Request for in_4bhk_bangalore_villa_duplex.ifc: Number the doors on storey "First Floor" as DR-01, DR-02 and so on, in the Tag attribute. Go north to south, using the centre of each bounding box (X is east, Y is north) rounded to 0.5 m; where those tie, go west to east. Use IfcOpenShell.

First a look at what the model holds.

```python
import ifcopenshell
import ifcopenshell.util.element
import ifcopenshell.util.placement

model = ifcopenshell.open("in_4bhk_bangalore_villa_duplex.ifc")
print(model.schema)
storey = next(s for s in model.by_type("IfcBuildingStorey") if s.Name == "First Floor")
doors = [e for e in ifcopenshell.util.element.get_decomposition(storey) if e.is_a("IfcDoor")]
for e in sorted(doors, key=lambda e: e.id()):
    origin = ifcopenshell.util.placement.get_local_placement(e.ObjectPlacement)[:3, 3]
    print(e.id(), e.Tag, e.Name, origin.round(2) + 0.0, sep=" | ")
```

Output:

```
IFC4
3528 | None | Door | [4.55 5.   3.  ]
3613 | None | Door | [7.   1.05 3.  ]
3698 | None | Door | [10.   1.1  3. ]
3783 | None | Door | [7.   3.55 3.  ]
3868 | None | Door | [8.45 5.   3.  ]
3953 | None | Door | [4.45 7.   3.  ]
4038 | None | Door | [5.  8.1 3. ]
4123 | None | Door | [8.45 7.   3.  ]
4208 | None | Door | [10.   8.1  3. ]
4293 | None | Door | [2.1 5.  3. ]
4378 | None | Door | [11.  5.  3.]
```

```python
import ifcopenshell
import ifcopenshell.geom
import ifcopenshell.util.element
import ifcopenshell.util.shape

model = ifcopenshell.open("in_4bhk_bangalore_villa_duplex.ifc")
settings = ifcopenshell.geom.settings()
settings.set("use-world-coords", True)


def centre(element):
    shape = ifcopenshell.geom.create_shape(settings, element)
    return ifcopenshell.util.shape.get_bbox_centroid(shape.geometry)


storey = next(s for s in model.by_type("IfcBuildingStorey") if s.Name == "First Floor")
doors = [e for e in ifcopenshell.util.element.get_decomposition(storey) if e.is_a("IfcDoor")]

# Insertion points can sit at a corner or the storey origin, so sort by the geometry (in metres).
centres = {e: centre(e) for e in doors}
doors.sort(key=lambda e: (-round(centres[e][1] / 0.5), centres[e][0]))

for i, e in enumerate(doors, start=1):
    number = f"DR-{i:02d}"
    e.Tag = number
    print(e.id(), number)

model.write("in_4bhk_bangalore_villa_duplex_rev.ifc")
```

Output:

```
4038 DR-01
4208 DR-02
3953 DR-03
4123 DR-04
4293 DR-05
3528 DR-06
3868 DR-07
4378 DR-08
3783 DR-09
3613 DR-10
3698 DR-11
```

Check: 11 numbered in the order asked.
